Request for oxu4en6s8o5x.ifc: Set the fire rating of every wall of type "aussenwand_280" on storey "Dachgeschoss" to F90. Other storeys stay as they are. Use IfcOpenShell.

First a look at what the model holds.

```python
import ifcopenshell
import ifcopenshell.util.element

model = ifcopenshell.open("oxu4en6s8o5x.ifc")
print(model.schema)
storey = next(s for s in model.by_type("IfcBuildingStorey") if s.Name == "Dachgeschoss")
walls = [e for e in ifcopenshell.util.element.get_decomposition(storey) if e.is_a("IfcWall")]
seen = {}
for e in walls:
    element_type = ifcopenshell.util.element.get_type(e)
    key = (element_type.Name if element_type != e and element_type else None, ifcopenshell.util.element.get_pset(e, "Pset_WallCommon", "FireRating"))
    seen[key] = seen.get(key, 0) + 1
for (name, value), count in sorted(seen.items(), key=str):
    print(count, "x", name, "|", value)
```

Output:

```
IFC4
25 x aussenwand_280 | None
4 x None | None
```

```python
import ifcopenshell
import ifcopenshell.api.pset
import ifcopenshell.util.element

model = ifcopenshell.open("oxu4en6s8o5x.ifc")

storey = next(s for s in model.by_type("IfcBuildingStorey") if s.Name == "Dachgeschoss")
walls = [e for e in ifcopenshell.util.element.get_decomposition(storey) if e.is_a("IfcWall")]

count = 0
for e in walls:
    element_type = ifcopenshell.util.element.get_type(e)
    if element_type in (None, e) or element_type.Name != "aussenwand_280":
        continue
    # add_pset returns the element's existing set when there is one.
    pset = ifcopenshell.api.pset.add_pset(model, product=e, name="Pset_WallCommon")
    ifcopenshell.api.pset.edit_pset(model, pset=pset, properties={"FireRating": "F90"})
    count += 1

print(count, "walls updated")

model.write("oxu4en6s8o5x_updated.ifc")
```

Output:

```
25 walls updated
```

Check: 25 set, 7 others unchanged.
